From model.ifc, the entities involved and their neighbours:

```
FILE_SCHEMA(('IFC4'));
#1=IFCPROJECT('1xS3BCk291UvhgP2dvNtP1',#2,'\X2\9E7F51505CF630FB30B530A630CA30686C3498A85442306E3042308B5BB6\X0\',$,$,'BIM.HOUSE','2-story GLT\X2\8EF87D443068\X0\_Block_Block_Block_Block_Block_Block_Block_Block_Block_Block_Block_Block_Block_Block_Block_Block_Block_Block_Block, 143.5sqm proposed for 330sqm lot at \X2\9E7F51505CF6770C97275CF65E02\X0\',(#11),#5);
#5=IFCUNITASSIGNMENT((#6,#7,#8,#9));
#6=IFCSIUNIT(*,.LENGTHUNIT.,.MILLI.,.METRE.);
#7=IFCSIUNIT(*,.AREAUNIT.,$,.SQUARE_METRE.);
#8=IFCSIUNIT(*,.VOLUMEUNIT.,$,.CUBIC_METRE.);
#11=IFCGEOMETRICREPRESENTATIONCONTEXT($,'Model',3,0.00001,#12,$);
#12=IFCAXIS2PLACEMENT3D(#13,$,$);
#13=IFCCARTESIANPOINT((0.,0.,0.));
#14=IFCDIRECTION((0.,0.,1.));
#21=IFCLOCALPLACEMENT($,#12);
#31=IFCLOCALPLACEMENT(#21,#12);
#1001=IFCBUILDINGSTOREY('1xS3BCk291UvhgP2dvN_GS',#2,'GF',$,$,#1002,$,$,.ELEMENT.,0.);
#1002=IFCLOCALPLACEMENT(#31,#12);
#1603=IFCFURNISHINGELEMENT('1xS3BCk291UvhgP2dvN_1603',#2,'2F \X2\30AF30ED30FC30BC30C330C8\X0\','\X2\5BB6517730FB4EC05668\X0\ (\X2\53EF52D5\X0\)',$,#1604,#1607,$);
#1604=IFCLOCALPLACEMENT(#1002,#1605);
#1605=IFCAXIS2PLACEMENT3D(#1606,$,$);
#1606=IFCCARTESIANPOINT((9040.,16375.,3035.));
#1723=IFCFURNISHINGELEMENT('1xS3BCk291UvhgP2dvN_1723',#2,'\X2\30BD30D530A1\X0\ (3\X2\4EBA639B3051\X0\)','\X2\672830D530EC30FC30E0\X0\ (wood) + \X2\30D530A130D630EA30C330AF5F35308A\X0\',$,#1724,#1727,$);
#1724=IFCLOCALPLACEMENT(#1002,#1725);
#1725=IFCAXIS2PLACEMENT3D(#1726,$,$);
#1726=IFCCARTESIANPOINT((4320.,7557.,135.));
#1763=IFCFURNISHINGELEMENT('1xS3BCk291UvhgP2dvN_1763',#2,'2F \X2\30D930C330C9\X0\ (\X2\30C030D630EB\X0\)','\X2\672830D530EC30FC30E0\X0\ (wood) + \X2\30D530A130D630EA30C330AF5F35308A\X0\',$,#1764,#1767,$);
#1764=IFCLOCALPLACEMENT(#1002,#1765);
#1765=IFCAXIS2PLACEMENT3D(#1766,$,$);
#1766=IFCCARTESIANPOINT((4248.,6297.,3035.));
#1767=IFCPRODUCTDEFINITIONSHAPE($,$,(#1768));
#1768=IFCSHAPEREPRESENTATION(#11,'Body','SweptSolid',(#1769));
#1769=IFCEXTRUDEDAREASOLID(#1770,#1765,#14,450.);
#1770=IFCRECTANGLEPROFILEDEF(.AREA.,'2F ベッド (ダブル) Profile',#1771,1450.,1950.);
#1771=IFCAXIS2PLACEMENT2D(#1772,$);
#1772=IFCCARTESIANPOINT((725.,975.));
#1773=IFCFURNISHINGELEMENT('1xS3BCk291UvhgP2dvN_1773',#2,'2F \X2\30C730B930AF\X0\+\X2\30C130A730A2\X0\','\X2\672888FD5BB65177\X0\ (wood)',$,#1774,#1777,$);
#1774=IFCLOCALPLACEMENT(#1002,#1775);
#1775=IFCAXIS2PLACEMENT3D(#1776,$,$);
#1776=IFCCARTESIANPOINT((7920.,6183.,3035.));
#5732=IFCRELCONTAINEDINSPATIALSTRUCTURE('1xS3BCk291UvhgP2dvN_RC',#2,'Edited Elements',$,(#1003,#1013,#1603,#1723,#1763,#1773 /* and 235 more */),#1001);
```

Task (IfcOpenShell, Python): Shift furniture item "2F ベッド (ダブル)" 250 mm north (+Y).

```python
import ifcopenshell
import ifcopenshell.api.geometry
import ifcopenshell.util.placement

model = ifcopenshell.open("model.ifc")

item = model.by_guid("1xS3BCk291UvhgP2dvN_1763")
matrix = ifcopenshell.util.placement.get_local_placement(item.ObjectPlacement)
matrix[1, 3] += 250.0
ifcopenshell.api.geometry.edit_object_placement(model, product=item, matrix=matrix, is_si=False)

print(ifcopenshell.util.placement.get_local_placement(item.ObjectPlacement).round(3) + 0.0)

model.write("model_rev.ifc")
```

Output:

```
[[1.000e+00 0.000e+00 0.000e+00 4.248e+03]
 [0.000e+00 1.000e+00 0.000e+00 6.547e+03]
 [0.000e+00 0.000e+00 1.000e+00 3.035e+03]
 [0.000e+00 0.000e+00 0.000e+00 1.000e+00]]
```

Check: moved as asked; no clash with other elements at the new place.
